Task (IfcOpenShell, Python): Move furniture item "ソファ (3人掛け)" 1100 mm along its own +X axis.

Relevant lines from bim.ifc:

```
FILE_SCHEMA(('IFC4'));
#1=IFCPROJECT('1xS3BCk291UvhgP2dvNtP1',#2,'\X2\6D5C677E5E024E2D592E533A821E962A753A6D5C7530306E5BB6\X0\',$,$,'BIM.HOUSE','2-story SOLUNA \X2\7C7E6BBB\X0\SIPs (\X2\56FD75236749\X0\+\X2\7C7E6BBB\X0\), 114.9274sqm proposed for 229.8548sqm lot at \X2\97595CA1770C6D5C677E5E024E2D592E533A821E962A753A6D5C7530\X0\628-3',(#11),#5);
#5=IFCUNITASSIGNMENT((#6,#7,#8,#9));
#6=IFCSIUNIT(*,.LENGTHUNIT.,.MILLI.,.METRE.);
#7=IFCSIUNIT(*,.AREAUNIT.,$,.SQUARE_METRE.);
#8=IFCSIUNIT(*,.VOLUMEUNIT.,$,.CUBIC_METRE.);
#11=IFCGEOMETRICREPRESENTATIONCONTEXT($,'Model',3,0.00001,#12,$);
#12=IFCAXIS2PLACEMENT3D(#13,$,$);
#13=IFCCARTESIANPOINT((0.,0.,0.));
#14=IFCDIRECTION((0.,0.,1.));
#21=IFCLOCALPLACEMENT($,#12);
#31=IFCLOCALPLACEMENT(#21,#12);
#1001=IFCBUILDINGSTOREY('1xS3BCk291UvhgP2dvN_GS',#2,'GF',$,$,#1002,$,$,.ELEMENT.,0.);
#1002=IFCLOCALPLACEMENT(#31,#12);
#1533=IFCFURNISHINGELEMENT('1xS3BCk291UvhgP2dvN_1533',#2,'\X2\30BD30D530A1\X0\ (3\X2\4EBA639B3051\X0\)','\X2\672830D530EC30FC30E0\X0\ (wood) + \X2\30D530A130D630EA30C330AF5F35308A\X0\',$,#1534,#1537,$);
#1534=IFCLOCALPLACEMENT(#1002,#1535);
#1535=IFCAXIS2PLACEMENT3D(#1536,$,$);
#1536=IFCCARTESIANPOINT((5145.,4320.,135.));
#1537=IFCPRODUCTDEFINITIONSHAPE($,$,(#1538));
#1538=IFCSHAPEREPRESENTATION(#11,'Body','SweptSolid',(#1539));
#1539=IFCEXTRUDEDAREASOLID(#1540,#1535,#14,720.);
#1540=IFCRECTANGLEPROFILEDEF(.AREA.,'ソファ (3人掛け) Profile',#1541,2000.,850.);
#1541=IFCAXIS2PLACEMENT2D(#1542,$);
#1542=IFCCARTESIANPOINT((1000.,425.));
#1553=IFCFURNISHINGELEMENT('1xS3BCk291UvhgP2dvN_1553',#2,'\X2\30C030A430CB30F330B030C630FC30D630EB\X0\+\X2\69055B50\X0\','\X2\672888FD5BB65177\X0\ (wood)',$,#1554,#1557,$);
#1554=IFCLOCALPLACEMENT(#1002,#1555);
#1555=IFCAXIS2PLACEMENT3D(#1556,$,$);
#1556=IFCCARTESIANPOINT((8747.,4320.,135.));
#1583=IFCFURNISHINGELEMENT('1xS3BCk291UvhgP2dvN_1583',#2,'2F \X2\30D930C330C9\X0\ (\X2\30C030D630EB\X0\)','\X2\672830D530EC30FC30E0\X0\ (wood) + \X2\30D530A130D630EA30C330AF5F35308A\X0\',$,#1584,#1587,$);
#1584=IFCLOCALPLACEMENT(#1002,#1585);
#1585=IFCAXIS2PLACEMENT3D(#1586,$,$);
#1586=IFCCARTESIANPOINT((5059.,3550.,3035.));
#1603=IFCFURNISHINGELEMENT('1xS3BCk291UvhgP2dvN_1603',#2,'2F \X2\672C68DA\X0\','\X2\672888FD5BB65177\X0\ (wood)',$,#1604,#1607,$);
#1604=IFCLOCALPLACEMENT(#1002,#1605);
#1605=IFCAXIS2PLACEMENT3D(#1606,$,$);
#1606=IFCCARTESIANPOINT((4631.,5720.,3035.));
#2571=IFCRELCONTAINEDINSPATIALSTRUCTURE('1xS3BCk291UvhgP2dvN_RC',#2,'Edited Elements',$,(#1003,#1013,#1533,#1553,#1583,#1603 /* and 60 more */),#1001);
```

```python
import ifcopenshell
import ifcopenshell.api.geometry
import ifcopenshell.util.placement

model = ifcopenshell.open("bim.ifc")

item = model.by_id(1533)
matrix = ifcopenshell.util.placement.get_local_placement(item.ObjectPlacement)
matrix[:3, 3] += matrix[:3, 0] * 1100.0
ifcopenshell.api.geometry.edit_object_placement(model, product=item, matrix=matrix, is_si=False)

print(ifcopenshell.util.placement.get_local_placement(item.ObjectPlacement).round(3) + 0.0)

model.write("bim_v2.ifc")
```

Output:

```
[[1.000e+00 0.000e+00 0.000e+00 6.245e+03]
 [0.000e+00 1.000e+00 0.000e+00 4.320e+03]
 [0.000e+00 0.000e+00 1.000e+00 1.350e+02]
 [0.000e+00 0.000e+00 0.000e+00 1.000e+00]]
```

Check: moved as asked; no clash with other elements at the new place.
